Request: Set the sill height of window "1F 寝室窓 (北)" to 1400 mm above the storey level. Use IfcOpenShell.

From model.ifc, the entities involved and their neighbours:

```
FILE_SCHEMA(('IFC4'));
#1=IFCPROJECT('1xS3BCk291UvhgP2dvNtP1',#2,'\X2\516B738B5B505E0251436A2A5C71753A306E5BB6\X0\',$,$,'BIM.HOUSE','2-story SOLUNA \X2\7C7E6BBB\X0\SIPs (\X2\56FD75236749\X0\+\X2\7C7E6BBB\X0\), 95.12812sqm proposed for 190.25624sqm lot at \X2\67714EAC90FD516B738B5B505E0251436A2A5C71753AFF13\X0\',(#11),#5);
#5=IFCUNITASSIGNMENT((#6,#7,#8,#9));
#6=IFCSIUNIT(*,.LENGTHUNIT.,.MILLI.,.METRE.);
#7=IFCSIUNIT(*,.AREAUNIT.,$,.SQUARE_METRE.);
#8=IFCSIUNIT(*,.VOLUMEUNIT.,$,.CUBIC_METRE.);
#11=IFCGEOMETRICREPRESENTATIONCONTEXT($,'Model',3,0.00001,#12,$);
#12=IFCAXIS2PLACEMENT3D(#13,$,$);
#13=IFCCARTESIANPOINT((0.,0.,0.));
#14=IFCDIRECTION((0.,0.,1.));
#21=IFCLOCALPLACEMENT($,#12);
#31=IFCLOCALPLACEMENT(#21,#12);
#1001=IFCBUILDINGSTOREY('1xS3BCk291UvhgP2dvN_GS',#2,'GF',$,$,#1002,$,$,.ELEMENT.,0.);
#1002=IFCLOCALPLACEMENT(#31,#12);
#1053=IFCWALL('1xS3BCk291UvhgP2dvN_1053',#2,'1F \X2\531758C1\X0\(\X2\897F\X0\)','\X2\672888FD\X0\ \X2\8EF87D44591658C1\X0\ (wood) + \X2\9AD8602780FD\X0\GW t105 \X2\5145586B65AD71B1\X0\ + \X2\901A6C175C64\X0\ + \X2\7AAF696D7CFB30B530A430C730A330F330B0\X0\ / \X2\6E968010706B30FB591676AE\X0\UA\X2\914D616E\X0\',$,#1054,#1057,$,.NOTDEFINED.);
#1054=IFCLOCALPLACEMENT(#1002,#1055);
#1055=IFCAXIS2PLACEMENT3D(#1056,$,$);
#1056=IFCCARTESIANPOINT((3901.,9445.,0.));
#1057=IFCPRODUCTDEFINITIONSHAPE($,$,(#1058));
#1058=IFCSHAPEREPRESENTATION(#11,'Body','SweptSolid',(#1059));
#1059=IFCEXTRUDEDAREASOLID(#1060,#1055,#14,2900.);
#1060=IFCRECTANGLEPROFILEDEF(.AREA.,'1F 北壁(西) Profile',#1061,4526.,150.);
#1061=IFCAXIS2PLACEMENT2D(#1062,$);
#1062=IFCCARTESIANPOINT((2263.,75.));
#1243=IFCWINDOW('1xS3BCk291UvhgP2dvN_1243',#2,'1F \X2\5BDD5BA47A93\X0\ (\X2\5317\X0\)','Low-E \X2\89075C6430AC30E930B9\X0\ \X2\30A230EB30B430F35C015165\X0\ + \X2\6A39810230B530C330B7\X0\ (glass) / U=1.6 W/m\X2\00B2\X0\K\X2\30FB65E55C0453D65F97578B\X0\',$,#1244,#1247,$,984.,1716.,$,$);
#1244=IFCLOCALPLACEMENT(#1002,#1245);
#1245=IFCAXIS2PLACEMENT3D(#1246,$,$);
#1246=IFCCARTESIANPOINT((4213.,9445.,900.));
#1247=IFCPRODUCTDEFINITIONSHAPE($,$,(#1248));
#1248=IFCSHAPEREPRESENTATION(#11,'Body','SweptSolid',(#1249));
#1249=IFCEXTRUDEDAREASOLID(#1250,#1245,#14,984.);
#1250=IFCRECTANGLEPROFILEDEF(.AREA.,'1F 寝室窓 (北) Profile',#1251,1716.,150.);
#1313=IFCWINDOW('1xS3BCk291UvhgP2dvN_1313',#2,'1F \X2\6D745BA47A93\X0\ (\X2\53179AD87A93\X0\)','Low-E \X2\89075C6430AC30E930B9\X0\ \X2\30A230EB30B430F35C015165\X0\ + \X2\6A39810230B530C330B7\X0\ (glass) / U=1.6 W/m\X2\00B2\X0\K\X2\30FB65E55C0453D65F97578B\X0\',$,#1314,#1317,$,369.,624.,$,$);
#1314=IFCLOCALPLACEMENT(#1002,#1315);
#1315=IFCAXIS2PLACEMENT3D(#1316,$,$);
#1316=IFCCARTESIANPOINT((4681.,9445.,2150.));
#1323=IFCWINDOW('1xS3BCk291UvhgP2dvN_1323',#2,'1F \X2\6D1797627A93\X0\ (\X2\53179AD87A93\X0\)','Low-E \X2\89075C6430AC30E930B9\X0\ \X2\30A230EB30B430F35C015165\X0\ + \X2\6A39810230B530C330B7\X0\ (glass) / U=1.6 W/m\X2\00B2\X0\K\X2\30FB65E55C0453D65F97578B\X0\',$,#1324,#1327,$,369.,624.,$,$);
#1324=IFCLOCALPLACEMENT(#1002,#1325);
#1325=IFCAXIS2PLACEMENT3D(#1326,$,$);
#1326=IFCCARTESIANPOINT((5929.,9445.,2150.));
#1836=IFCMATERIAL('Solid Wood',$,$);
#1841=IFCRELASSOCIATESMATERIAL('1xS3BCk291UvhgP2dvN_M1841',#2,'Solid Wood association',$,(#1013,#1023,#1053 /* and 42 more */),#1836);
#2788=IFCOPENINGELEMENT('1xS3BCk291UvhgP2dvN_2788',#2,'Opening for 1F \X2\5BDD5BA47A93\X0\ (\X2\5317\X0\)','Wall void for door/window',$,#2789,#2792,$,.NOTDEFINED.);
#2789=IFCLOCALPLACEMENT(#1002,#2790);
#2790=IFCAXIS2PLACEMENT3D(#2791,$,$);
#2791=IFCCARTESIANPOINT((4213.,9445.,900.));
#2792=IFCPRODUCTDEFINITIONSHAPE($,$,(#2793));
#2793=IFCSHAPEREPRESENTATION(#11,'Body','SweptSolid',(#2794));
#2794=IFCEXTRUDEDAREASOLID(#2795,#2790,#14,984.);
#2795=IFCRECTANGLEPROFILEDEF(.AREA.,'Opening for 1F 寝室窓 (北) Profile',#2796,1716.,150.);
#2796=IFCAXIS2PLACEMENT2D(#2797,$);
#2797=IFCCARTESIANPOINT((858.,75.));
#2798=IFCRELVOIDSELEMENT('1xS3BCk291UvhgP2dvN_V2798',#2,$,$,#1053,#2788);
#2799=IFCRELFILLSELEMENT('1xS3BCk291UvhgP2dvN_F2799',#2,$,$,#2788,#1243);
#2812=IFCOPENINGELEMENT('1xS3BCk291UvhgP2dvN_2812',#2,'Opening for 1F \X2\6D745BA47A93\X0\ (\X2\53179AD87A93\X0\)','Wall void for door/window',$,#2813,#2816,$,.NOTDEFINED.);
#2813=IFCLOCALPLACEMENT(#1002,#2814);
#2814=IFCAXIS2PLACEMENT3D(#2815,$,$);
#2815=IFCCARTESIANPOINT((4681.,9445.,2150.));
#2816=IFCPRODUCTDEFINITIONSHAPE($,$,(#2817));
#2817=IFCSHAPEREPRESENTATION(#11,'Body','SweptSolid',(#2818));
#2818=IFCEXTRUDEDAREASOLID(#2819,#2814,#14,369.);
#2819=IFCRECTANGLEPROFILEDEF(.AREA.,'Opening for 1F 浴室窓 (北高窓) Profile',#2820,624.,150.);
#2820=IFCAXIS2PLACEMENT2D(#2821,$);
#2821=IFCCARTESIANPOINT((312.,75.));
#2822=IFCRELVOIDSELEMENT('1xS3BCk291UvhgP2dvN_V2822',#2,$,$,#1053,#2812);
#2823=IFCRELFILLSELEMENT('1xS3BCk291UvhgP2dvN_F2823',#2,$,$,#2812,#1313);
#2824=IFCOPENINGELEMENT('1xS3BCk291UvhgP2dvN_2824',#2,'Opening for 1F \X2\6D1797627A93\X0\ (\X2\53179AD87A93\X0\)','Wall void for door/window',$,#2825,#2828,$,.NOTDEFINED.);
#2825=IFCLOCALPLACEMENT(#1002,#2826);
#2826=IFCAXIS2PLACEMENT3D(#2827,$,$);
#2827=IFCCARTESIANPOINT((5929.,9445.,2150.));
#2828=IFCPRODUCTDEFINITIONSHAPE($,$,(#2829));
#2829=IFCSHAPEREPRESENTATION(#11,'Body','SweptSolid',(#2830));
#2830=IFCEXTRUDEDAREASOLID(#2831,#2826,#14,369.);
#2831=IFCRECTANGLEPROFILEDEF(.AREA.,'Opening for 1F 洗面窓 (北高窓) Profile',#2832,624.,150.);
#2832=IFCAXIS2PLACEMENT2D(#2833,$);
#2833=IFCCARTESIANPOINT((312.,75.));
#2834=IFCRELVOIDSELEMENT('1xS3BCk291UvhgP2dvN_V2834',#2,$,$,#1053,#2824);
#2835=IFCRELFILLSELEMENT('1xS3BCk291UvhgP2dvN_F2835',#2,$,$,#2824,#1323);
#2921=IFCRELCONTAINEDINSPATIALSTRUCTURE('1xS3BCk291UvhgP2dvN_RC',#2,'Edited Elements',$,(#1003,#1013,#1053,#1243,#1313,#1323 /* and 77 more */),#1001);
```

```python
import numpy as np
import ifcopenshell
import ifcopenshell.api.geometry
import ifcopenshell.geom
import ifcopenshell.util.element
import ifcopenshell.util.placement
import ifcopenshell.util.shape
import ifcopenshell.util.unit

model = ifcopenshell.open("model.ifc")
unit_scale = ifcopenshell.util.unit.calculate_unit_scale(model)

window = model.by_guid("1xS3BCk291UvhgP2dvN_1243")
opening = window.FillsVoids[0].RelatingOpeningElement
storey = ifcopenshell.util.element.get_container(window, ifc_class="IfcBuildingStorey")
level = ifcopenshell.util.placement.get_local_placement(storey.ObjectPlacement)[2, 3]

# The opening's origin need not be at the sill, so measure its lowest point.
shape = ifcopenshell.geom.create_shape(ifcopenshell.geom.settings(), opening)
bottom = ifcopenshell.util.shape.get_shape_bottom_elevation(shape, shape.geometry) / unit_scale
dz = level + 1400.0 - bottom

shift = np.array([0.0, 0.0, dz])
# The window is not placed relative to its opening, so move both.
for product in (opening, window):
    matrix = ifcopenshell.util.placement.get_local_placement(product.ObjectPlacement)
    matrix[:3, 3] += shift
    ifcopenshell.api.geometry.edit_object_placement(model, product=product, matrix=matrix, is_si=False)

print(f"moved by {dz * unit_scale:+.3f} m")

model.write("model_v2.ifc")
```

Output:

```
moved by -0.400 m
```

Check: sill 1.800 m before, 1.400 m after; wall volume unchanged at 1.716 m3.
